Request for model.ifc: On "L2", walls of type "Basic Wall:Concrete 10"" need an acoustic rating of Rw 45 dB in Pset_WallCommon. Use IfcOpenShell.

First a look at what the model holds.

```python
import ifcopenshell
import ifcopenshell.util.element

model = ifcopenshell.open("model.ifc")
print(model.schema)
storey = next(s for s in model.by_type("IfcBuildingStorey") if s.Name == "L2")
walls = [e for e in ifcopenshell.util.element.get_decomposition(storey) if e.is_a("IfcWall")]
seen = {}
for e in walls:
    element_type = ifcopenshell.util.element.get_type(e)
    key = (element_type.Name if element_type != e and element_type else None, ifcopenshell.util.element.get_pset(e, "Pset_WallCommon", "AcousticRating"))
    seen[key] = seen.get(key, 0) + 1
for (name, value), count in sorted(seen.items(), key=str):
    print(count, "x", name, "|", value)
```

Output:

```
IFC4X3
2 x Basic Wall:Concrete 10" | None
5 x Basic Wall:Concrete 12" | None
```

```python
import ifcopenshell
import ifcopenshell.api.pset
import ifcopenshell.util.element

model = ifcopenshell.open("model.ifc")

storey = next(s for s in model.by_type("IfcBuildingStorey") if s.Name == "L2")
walls = [e for e in ifcopenshell.util.element.get_decomposition(storey) if e.is_a("IfcWall")]

count = 0
for e in walls:
    element_type = ifcopenshell.util.element.get_type(e)
    if element_type in (None, e) or element_type.Name != 'Basic Wall:Concrete 10"':
        continue
    # add_pset returns the element's existing set when there is one.
    pset = ifcopenshell.api.pset.add_pset(model, product=e, name="Pset_WallCommon")
    ifcopenshell.api.pset.edit_pset(model, pset=pset, properties={"AcousticRating": "Rw 45 dB"})
    count += 1

print(count, "walls updated")

model.write("model-out.ifc")
```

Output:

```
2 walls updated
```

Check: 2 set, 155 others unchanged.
